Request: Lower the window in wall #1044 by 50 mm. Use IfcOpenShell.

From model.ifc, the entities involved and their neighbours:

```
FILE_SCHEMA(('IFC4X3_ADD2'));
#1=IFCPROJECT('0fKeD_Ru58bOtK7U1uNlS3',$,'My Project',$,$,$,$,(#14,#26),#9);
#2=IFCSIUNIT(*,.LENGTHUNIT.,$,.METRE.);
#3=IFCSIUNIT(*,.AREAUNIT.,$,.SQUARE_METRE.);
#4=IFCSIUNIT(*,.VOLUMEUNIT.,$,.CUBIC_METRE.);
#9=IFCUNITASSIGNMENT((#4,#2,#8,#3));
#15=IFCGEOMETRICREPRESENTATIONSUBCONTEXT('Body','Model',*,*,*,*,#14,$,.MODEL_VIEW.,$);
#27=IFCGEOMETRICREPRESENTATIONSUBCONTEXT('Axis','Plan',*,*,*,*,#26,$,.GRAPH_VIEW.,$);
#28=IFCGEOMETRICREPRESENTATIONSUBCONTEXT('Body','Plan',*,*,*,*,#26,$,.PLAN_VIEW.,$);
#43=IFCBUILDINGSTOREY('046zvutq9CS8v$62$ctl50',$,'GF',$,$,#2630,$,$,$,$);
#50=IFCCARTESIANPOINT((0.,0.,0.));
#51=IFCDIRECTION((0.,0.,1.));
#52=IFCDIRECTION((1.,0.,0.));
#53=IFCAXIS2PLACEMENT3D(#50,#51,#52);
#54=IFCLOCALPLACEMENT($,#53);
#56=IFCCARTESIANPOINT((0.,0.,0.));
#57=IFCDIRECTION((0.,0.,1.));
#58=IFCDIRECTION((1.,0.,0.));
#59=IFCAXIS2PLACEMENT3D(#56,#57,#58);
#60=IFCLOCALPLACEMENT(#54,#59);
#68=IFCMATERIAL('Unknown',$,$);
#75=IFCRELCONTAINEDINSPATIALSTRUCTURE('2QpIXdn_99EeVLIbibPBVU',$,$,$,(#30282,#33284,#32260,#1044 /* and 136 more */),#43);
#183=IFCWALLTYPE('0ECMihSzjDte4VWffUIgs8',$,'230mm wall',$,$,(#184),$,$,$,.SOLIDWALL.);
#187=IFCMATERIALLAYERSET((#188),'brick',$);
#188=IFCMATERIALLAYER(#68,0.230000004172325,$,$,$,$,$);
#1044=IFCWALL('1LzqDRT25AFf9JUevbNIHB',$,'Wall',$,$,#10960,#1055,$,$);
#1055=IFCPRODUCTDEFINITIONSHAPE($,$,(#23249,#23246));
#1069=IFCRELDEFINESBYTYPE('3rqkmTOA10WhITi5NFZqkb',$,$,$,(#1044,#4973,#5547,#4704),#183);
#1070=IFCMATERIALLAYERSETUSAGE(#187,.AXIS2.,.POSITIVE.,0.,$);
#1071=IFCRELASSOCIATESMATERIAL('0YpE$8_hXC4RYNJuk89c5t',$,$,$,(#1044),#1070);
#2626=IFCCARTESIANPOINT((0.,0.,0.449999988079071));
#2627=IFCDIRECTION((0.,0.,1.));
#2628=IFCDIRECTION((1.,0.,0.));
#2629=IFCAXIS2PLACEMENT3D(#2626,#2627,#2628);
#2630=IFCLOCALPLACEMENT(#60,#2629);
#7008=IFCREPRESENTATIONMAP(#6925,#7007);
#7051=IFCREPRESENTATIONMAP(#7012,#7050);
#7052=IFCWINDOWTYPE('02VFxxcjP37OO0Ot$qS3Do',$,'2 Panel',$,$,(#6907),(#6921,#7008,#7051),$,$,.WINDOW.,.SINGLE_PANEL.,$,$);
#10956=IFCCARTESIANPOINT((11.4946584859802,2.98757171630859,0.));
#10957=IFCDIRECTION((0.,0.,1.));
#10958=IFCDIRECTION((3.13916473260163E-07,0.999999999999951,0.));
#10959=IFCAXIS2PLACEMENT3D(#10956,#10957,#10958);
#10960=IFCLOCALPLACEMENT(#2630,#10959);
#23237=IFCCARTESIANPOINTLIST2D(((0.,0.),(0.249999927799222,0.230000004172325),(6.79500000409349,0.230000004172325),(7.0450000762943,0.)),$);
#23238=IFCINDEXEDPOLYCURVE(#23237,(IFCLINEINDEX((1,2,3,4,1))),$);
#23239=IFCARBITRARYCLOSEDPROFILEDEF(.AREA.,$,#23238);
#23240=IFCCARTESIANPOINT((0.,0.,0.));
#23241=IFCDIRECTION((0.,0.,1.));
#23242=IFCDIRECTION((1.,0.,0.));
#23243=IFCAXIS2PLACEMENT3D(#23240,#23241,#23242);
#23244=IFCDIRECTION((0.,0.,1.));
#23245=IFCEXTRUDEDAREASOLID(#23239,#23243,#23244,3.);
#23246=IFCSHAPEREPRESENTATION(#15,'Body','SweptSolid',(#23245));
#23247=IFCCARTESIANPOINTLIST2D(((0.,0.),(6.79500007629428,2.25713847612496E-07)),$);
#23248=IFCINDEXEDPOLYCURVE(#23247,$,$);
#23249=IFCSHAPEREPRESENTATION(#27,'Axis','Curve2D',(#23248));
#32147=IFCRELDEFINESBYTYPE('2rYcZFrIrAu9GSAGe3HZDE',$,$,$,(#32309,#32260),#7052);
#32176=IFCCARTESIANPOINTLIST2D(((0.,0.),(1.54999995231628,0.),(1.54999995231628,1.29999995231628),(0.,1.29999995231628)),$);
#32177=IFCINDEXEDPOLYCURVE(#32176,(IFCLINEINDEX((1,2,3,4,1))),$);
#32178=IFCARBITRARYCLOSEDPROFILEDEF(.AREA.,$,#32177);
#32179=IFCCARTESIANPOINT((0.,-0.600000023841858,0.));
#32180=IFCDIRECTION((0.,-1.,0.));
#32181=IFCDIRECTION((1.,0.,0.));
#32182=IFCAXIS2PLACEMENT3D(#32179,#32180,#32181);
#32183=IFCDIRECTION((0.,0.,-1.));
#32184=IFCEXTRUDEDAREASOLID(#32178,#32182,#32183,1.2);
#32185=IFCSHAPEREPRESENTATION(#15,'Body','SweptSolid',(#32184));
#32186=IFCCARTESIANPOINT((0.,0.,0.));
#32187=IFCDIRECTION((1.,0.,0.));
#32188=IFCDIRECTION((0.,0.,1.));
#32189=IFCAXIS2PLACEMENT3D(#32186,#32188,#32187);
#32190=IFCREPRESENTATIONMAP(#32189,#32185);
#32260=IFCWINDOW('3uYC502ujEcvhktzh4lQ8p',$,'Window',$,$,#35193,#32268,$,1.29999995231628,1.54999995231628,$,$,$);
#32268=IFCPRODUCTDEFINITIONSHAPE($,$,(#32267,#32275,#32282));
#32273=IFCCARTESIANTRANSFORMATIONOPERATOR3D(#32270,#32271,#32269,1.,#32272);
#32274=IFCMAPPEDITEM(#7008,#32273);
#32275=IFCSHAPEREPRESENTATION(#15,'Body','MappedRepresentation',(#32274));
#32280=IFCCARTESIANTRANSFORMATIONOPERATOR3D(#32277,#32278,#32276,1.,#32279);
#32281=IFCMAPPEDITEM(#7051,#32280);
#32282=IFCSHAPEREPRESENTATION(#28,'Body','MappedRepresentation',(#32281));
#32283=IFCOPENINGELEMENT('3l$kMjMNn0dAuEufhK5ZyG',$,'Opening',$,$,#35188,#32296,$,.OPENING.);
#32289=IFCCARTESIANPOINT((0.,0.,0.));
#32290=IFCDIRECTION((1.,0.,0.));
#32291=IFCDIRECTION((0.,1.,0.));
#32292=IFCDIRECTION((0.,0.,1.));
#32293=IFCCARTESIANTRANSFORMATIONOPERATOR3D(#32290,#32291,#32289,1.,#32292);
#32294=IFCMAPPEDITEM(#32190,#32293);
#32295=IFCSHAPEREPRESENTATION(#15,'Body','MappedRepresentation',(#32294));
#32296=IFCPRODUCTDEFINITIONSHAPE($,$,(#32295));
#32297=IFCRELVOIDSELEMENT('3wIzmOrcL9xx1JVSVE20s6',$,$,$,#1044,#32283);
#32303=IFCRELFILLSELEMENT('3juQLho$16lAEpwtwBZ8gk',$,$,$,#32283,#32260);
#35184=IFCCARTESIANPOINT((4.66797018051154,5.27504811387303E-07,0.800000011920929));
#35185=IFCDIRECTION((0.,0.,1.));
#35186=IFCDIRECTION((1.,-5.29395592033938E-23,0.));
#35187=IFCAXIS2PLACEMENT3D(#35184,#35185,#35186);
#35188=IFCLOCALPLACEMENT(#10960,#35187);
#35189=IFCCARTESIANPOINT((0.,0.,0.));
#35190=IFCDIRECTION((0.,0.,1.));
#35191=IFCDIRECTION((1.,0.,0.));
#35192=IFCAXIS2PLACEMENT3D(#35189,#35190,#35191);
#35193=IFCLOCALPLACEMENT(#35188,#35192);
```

```python
import numpy as np
import ifcopenshell
import ifcopenshell.api.geometry
import ifcopenshell.util.placement
import ifcopenshell.util.unit

model = ifcopenshell.open("model.ifc")
unit_scale = ifcopenshell.util.unit.calculate_unit_scale(model)

window = model.by_id(32260)
opening = window.FillsVoids[0].RelatingOpeningElement
dz = -0.05

shift = np.array([0.0, 0.0, dz])
# The window is placed relative to its opening, so it follows when the opening moves.
matrix = ifcopenshell.util.placement.get_local_placement(opening.ObjectPlacement)
matrix[:3, 3] += shift
ifcopenshell.api.geometry.edit_object_placement(
    model, product=opening, matrix=matrix, is_si=False, should_transform_children=True
)

print(f"moved by {dz * unit_scale:+.3f} m")

model.write("model_v2.ifc")
```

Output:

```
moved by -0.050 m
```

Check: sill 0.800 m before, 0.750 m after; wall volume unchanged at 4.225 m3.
